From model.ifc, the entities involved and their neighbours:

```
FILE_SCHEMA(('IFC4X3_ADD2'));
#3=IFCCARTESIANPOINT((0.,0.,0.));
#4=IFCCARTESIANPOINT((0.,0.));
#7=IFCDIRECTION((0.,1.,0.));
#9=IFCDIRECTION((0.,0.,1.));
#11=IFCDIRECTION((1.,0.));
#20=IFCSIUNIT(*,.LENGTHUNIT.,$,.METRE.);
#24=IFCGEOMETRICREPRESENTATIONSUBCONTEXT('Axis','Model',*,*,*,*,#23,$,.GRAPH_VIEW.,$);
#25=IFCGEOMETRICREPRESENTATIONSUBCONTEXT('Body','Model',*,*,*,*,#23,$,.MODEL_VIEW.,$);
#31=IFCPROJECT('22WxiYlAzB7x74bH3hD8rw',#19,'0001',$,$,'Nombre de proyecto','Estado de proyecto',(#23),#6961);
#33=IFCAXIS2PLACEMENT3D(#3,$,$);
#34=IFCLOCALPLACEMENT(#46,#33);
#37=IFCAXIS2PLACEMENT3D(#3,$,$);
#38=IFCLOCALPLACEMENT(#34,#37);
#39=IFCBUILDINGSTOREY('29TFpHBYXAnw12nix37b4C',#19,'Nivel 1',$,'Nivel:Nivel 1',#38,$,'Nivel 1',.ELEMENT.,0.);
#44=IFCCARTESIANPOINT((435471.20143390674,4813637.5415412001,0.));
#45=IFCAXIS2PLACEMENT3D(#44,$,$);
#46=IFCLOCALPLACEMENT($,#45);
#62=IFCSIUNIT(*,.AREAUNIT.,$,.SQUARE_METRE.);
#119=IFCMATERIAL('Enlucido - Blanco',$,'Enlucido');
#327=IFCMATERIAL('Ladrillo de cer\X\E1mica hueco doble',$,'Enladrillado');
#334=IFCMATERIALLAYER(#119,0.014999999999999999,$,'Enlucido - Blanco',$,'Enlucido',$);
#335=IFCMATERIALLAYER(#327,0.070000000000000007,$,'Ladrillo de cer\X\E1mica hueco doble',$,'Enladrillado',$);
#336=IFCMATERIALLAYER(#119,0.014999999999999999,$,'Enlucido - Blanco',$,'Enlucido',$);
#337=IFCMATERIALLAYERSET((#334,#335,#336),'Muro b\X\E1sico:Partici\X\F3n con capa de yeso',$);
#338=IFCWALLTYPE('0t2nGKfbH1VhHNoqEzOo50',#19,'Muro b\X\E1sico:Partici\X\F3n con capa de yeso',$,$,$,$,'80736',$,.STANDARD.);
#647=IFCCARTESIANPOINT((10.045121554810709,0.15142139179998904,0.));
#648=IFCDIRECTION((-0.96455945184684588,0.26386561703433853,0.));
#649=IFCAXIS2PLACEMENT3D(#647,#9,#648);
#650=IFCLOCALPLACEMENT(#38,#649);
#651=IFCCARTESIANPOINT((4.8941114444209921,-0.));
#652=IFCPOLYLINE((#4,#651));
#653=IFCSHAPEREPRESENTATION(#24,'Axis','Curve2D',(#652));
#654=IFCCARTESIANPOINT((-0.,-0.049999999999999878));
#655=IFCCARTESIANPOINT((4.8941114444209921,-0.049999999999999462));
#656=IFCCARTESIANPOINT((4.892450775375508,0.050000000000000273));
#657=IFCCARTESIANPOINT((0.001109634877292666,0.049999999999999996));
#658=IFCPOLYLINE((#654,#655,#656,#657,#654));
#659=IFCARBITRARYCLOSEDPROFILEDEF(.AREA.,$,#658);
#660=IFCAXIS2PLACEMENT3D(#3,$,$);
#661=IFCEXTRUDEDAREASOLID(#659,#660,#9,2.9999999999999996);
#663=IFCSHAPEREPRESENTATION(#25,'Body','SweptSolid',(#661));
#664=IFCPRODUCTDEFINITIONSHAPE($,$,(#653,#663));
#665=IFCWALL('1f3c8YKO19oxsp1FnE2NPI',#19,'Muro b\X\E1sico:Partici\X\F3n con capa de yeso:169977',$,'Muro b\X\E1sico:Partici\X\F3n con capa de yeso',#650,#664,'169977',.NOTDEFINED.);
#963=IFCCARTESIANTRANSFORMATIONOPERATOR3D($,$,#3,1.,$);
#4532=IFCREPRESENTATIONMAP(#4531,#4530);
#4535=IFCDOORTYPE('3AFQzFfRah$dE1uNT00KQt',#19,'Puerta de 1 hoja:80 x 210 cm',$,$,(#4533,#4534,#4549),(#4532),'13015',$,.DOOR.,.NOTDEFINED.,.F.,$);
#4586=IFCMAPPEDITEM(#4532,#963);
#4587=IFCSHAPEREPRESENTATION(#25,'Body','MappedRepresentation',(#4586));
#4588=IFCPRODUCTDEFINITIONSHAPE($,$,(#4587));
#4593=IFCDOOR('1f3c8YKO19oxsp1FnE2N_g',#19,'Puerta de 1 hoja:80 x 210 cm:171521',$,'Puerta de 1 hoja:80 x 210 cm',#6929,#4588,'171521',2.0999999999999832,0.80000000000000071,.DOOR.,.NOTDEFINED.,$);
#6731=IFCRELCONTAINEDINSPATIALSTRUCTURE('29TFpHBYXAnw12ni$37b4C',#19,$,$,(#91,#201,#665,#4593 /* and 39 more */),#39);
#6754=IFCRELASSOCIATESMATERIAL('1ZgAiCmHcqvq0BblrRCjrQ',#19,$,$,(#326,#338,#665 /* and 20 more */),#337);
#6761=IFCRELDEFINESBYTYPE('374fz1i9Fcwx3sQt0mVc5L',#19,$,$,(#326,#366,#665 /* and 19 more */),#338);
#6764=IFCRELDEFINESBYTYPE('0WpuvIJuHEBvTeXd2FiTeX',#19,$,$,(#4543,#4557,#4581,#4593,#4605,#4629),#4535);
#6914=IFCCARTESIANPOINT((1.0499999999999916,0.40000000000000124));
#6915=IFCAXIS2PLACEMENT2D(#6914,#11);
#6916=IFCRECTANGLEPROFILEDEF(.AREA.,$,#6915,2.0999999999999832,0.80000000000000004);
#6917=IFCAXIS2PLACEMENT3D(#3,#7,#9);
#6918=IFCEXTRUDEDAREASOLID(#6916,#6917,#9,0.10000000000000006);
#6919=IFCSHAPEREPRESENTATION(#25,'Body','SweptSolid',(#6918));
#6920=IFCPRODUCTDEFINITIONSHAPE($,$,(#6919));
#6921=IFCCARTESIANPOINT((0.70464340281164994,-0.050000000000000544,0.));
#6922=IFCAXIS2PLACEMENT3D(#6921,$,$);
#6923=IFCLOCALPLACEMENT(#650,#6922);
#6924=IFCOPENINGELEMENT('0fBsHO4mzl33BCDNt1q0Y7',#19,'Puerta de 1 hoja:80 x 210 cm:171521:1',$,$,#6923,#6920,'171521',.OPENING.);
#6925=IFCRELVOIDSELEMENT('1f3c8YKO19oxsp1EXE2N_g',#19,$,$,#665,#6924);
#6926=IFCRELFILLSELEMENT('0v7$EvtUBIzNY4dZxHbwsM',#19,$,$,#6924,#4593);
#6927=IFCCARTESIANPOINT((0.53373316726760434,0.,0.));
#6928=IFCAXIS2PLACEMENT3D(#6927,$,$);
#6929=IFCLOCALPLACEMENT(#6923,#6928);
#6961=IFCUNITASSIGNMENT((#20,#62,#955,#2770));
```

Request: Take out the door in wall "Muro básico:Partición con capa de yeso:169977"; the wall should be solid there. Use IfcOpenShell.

```python
import ifcopenshell
import ifcopenshell.api.feature
import ifcopenshell.api.root
import ifcopenshell.geom
import ifcopenshell.util.shape

model = ifcopenshell.open("model.ifc")
settings = ifcopenshell.geom.settings()


def volume(element):
    """Net volume in cubic metres, openings subtracted."""
    shape = ifcopenshell.geom.create_shape(settings, element)
    return ifcopenshell.util.shape.get_volume(shape.geometry)


door = model.by_guid("1f3c8YKO19oxsp1FnE2N_g")
opening = door.FillsVoids[0].RelatingOpeningElement
wall = opening.VoidsElements[0].RelatingBuildingElement
before = volume(wall)

ifcopenshell.api.root.remove_product(model, product=door)
ifcopenshell.api.feature.remove_feature(model, feature=opening)

after = volume(wall)

print(f"wall volume {before:.3f} -> {after:.3f} m3")

model.write("model_rev.ifc")
```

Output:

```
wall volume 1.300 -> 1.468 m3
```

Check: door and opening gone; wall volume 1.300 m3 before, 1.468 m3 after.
